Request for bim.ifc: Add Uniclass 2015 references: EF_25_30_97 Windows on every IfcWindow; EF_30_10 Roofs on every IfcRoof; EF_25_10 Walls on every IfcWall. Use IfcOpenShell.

First a look at what the model holds.

```python
import ifcopenshell

model = ifcopenshell.open("bim.ifc")
print(model.schema)
print("classifications:", [c.Name for c in model.by_type("IfcClassification")])
for ifc_class in ("IfcDoor", "IfcRoof", "IfcStair", "IfcWall", "IfcWindow"):
    print(ifc_class, len(model.by_type(ifc_class)))
```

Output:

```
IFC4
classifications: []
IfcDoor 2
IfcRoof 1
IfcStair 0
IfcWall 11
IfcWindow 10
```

```python
import ifcopenshell
import ifcopenshell.api.classification

model = ifcopenshell.open("bim.ifc")

system = ifcopenshell.api.classification.add_classification(model, classification="Uniclass 2015")

codes = {
    "IfcWindow": ("EF_25_30_97", "Windows"),
    "IfcRoof": ("EF_30_10", "Roofs"),
    "IfcWall": ("EF_25_10", "Walls"),
}
for ifc_class, (code, name) in codes.items():
    products = model.by_type(ifc_class)
    ifcopenshell.api.classification.add_reference(
        model, products=products, classification=system, identification=code, name=name
    )
    print(code, len(products))

model.write("bim_edited.ifc")
```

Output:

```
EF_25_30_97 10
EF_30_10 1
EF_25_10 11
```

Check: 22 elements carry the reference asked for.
